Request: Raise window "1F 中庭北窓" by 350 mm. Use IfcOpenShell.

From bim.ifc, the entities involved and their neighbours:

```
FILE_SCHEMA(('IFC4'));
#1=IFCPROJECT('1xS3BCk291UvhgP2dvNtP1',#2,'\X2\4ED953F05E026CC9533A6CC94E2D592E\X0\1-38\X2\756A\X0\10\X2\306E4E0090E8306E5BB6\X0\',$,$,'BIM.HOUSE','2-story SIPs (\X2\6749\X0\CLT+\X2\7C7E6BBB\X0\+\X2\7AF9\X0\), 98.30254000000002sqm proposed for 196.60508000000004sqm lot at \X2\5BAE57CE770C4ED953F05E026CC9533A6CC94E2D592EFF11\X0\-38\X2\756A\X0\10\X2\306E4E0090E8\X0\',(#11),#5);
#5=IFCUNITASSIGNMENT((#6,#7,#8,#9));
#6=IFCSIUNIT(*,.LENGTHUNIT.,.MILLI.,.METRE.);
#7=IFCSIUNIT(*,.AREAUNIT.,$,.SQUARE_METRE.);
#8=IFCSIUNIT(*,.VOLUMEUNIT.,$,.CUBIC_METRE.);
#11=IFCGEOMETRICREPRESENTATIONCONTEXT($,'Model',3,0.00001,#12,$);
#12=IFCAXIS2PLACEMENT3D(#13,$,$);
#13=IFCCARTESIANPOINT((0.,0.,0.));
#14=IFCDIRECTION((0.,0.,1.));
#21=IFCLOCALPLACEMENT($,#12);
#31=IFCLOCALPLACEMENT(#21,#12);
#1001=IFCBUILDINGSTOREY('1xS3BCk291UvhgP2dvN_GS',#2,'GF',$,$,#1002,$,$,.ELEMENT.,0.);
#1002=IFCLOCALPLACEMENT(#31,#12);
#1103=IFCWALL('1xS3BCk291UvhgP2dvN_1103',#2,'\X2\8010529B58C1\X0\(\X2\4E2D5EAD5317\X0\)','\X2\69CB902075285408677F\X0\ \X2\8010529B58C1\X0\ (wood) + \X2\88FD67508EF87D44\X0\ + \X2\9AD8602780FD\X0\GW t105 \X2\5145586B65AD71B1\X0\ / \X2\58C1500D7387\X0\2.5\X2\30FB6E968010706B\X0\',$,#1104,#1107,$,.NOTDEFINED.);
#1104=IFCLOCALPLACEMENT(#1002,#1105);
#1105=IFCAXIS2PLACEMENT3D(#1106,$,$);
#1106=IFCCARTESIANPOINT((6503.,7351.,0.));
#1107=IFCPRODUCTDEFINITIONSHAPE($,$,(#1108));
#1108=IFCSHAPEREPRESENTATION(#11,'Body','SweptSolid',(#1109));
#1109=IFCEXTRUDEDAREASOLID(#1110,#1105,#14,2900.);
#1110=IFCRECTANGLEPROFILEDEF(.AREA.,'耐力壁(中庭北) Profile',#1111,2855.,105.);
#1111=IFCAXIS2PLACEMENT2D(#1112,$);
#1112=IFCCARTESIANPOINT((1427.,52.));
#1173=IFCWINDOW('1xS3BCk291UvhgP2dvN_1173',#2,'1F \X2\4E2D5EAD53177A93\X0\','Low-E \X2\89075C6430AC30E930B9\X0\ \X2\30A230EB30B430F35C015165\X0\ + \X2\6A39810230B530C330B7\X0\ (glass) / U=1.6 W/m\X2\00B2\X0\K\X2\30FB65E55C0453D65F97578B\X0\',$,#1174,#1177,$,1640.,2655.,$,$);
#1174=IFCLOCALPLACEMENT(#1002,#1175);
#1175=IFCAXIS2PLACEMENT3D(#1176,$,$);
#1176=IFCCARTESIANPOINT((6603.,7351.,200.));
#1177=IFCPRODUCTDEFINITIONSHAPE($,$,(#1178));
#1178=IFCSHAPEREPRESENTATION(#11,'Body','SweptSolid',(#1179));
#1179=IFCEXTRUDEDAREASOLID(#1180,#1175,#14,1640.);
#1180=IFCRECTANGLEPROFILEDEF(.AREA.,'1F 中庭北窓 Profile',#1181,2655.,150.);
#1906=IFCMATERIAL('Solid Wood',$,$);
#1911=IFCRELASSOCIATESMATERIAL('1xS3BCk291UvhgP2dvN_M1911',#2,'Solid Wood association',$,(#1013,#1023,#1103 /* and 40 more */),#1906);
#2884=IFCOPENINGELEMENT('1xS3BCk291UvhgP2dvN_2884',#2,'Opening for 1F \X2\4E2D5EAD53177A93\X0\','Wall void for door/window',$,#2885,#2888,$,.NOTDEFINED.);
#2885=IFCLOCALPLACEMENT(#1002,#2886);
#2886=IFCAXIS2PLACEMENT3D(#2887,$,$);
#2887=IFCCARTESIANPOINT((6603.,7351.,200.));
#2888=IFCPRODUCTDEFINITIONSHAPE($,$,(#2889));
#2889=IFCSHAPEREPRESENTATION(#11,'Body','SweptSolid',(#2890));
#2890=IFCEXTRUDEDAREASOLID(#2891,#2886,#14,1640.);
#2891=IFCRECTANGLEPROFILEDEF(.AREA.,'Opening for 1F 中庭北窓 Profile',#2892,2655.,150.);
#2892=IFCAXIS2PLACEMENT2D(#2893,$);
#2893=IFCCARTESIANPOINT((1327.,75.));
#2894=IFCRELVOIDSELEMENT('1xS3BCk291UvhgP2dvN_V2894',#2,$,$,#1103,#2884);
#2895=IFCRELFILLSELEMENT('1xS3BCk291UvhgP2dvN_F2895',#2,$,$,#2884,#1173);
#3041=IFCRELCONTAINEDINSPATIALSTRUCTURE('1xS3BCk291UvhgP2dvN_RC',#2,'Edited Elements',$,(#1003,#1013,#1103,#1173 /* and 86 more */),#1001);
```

```python
import numpy as np
import ifcopenshell
import ifcopenshell.api.geometry
import ifcopenshell.util.placement
import ifcopenshell.util.unit

model = ifcopenshell.open("bim.ifc")
unit_scale = ifcopenshell.util.unit.calculate_unit_scale(model)

window = model.by_id(1173)
opening = window.FillsVoids[0].RelatingOpeningElement
dz = 350.0

shift = np.array([0.0, 0.0, dz])
# The window is not placed relative to its opening, so move both.
for product in (opening, window):
    matrix = ifcopenshell.util.placement.get_local_placement(product.ObjectPlacement)
    matrix[:3, 3] += shift
    ifcopenshell.api.geometry.edit_object_placement(model, product=product, matrix=matrix, is_si=False)

print(f"moved by {dz * unit_scale:+.3f} m")

model.write("bim_v2.ifc")
```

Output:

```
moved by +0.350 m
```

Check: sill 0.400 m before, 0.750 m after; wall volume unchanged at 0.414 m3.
